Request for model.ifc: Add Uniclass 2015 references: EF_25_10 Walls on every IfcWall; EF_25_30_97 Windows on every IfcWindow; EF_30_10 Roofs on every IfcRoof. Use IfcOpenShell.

First a look at what the model holds.

```python
import ifcopenshell

model = ifcopenshell.open("model.ifc")
print(model.schema)
print("classifications:", [c.Name for c in model.by_type("IfcClassification")])
for ifc_class in ("IfcDoor", "IfcRoof", "IfcStair", "IfcWall", "IfcWindow"):
    print(ifc_class, len(model.by_type(ifc_class)))
```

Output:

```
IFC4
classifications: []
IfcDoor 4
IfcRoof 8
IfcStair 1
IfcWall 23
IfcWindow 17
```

```python
import ifcopenshell
import ifcopenshell.api.classification

model = ifcopenshell.open("model.ifc")

system = ifcopenshell.api.classification.add_classification(model, classification="Uniclass 2015")

codes = {
    "IfcWall": ("EF_25_10", "Walls"),
    "IfcWindow": ("EF_25_30_97", "Windows"),
    "IfcRoof": ("EF_30_10", "Roofs"),
}
for ifc_class, (code, name) in codes.items():
    products = model.by_type(ifc_class)
    ifcopenshell.api.classification.add_reference(
        model, products=products, classification=system, identification=code, name=name
    )
    print(code, len(products))

model.write("model_rev.ifc")
```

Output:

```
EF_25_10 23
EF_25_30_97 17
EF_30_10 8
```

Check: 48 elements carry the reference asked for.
